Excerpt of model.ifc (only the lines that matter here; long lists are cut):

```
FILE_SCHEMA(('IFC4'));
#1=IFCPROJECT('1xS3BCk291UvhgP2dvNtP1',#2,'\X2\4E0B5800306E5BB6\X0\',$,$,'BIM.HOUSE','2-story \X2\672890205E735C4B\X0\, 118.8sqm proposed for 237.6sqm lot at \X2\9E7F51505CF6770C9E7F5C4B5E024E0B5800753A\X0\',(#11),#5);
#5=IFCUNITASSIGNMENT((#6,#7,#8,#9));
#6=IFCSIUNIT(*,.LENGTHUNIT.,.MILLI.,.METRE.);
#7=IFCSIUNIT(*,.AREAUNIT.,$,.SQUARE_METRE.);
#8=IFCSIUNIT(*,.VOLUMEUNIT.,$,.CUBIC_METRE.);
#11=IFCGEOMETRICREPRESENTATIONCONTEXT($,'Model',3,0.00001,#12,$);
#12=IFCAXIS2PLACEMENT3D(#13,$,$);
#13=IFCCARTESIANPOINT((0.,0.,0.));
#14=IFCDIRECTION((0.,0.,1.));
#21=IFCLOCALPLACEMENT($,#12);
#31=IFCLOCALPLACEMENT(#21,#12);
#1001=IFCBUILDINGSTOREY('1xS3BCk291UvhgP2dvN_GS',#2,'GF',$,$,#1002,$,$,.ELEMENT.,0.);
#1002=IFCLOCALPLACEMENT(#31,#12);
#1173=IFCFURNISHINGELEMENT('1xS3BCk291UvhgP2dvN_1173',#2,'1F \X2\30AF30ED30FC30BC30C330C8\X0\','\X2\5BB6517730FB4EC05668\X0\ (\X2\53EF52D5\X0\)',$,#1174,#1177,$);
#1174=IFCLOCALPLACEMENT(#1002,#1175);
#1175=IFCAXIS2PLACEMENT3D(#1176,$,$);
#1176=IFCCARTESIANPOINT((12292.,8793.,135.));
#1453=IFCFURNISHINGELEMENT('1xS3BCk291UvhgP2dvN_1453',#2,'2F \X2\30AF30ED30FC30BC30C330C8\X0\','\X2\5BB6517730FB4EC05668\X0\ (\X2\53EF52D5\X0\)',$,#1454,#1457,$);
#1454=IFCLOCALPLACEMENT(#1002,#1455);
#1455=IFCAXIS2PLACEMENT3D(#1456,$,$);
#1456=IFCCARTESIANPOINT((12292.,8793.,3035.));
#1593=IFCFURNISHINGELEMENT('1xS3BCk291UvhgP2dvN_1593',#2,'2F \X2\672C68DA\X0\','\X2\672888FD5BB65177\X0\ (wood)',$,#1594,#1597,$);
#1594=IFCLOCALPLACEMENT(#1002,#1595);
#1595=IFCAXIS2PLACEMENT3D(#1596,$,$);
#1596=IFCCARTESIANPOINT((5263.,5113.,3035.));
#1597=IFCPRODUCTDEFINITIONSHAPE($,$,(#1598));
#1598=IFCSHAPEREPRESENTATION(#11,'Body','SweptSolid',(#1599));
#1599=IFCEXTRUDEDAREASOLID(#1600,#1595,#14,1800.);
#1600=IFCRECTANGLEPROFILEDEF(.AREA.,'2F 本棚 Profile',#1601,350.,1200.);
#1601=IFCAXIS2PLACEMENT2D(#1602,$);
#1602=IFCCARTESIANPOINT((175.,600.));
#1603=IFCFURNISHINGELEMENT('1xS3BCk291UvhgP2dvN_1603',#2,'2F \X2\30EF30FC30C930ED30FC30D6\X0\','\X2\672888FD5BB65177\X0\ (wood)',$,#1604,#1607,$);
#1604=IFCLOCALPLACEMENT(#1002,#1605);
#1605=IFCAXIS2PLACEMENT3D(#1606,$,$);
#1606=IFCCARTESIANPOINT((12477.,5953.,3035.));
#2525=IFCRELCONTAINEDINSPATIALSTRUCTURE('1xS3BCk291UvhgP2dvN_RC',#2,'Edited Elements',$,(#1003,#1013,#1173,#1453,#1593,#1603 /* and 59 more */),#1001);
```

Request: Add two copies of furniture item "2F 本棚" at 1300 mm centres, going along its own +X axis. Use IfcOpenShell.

```python
import ifcopenshell
import ifcopenshell.api.geometry
import ifcopenshell.api.root
import ifcopenshell.util.element
import ifcopenshell.util.placement
import ifcopenshell.util.unit

model = ifcopenshell.open("model.ifc")
unit_scale = ifcopenshell.util.unit.calculate_unit_scale(model)


def reuse_history(source, copy):
    """copy_class also copies each property set's owner history, people and application; keep the originals."""
    for rel in copy.IsDefinedBy:
        if rel.is_a("IfcRelDefinesByProperties") and (history := rel.RelatingPropertyDefinition.OwnerHistory):
            rel.RelatingPropertyDefinition.OwnerHistory = source.OwnerHistory
            ifcopenshell.util.element.remove_deep2(model, history)


source = model.by_guid("1xS3BCk291UvhgP2dvN_1593")
base = ifcopenshell.util.placement.get_local_placement(source.ObjectPlacement)
step = base[:3, 0] * 1.3 / unit_scale

for i in range(1, 3):
    copy = ifcopenshell.api.root.copy_class(model, product=source)
    copy.Representation = ifcopenshell.util.element.copy_deep(
        model, source.Representation, exclude=["IfcGeometricRepresentationContext", "IfcRepresentationMap"]
    )
    reuse_history(source, copy)
    matrix = base.copy()
    matrix[:3, 3] += i * step
    print("added at", matrix[:3, 3].round(3) + 0.0)
    ifcopenshell.api.geometry.edit_object_placement(model, product=copy, matrix=matrix, is_si=False)

model.write("model_updated.ifc")
```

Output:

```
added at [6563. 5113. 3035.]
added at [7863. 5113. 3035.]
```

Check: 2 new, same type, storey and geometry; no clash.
